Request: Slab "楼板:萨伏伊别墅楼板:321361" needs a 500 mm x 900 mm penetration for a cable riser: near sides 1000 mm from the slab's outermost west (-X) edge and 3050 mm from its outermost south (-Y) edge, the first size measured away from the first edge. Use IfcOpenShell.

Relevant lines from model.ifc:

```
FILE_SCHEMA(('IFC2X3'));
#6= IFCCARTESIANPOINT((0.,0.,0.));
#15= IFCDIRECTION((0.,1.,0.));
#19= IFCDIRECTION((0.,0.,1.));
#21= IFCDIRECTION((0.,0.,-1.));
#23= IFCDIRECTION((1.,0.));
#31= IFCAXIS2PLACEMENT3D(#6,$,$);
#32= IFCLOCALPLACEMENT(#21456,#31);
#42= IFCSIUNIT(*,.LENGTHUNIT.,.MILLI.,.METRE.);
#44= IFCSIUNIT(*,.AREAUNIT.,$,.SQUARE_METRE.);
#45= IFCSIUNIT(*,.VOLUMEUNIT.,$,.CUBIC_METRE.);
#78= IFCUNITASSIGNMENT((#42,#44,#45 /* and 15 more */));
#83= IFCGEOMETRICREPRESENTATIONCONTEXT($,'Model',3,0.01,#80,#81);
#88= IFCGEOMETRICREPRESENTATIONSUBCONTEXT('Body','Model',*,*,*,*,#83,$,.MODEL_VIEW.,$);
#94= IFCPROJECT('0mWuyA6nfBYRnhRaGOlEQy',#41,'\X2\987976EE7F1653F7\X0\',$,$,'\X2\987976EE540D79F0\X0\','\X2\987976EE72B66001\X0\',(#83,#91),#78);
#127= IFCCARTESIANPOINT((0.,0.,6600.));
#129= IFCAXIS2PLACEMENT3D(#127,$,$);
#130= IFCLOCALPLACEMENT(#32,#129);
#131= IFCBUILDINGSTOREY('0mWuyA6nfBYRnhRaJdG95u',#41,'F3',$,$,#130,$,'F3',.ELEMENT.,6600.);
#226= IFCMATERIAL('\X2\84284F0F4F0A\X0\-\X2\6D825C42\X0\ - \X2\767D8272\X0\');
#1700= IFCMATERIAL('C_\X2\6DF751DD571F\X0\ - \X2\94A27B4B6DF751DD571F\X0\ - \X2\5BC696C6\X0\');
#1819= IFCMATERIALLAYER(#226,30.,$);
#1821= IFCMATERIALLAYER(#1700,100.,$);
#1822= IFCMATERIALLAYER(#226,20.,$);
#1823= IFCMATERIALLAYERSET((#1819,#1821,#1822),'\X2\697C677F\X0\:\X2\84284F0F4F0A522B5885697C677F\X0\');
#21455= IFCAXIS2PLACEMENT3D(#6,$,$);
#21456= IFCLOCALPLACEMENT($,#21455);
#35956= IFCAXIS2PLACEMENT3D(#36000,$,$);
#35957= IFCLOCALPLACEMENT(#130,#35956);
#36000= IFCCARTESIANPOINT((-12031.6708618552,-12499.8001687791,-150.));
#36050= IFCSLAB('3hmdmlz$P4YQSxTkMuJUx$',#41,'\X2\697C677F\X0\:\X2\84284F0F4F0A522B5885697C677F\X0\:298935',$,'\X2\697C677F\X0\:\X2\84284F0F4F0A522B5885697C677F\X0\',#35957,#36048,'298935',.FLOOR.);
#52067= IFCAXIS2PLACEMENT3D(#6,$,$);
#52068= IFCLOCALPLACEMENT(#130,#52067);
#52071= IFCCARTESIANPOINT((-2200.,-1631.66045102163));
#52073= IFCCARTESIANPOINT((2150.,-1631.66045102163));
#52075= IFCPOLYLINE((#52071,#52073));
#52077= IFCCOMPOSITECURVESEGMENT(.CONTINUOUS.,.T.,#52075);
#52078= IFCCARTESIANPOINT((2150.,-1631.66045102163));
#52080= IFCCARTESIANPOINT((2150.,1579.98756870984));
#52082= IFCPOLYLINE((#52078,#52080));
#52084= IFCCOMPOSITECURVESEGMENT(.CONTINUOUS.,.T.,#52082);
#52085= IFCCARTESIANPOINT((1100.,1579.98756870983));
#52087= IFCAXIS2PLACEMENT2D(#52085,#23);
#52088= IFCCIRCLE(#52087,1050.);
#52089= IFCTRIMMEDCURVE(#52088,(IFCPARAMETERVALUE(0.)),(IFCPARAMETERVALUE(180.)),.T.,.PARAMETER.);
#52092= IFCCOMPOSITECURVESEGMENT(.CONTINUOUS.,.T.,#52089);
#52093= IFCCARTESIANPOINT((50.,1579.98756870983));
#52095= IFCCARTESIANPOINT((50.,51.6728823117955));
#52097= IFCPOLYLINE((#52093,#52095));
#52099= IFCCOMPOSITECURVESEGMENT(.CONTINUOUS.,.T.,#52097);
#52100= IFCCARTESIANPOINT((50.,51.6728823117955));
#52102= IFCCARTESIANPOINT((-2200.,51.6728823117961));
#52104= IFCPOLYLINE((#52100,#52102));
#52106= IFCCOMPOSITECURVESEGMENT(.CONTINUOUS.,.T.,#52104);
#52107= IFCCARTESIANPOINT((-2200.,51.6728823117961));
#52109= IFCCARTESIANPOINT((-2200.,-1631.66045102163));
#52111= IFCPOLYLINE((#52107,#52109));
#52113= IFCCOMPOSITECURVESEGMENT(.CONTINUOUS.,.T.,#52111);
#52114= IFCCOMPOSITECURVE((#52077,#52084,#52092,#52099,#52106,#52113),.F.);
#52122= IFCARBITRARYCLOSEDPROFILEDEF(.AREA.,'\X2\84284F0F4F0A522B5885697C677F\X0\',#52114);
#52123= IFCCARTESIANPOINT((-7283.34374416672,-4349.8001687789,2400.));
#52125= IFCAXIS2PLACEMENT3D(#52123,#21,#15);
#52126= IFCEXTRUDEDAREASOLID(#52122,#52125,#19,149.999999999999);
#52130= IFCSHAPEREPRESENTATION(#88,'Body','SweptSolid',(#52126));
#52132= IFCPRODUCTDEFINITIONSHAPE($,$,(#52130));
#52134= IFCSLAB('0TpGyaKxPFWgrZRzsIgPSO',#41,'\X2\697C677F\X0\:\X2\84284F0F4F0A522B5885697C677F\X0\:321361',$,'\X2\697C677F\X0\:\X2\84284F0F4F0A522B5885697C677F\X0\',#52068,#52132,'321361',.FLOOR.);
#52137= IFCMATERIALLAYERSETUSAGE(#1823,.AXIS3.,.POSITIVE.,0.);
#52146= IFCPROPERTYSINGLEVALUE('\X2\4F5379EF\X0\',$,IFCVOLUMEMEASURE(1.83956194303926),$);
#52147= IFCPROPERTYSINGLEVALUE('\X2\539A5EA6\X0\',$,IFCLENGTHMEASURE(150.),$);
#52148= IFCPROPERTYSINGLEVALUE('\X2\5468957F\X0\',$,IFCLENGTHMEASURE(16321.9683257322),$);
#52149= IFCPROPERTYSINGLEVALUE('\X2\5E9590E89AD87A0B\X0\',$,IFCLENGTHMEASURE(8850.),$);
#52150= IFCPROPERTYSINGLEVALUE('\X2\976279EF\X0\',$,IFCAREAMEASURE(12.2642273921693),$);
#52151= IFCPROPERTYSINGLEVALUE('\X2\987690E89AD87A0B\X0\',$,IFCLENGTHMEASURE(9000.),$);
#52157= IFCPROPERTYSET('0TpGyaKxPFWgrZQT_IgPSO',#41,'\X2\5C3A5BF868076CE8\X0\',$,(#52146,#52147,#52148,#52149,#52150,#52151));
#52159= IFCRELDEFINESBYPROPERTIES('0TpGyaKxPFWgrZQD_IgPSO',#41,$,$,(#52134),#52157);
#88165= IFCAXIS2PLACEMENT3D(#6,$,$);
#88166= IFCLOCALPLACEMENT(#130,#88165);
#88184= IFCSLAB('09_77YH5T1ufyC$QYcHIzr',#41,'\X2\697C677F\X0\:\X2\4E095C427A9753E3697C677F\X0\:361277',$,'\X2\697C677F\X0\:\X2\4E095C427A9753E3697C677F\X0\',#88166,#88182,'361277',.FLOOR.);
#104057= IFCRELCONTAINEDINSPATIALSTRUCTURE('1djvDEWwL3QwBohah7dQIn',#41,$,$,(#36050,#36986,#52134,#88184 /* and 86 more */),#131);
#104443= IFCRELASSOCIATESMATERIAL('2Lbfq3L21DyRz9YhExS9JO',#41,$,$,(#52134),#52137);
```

```python
import numpy as np
import ifcopenshell
import ifcopenshell.api.feature
import ifcopenshell.api.geometry
import ifcopenshell.api.pset
import ifcopenshell.api.root
import ifcopenshell.geom
import ifcopenshell.util.element
import ifcopenshell.util.placement
import ifcopenshell.util.representation
import ifcopenshell.util.shape
import ifcopenshell.util.unit

model = ifcopenshell.open("model.ifc")
unit_scale = ifcopenshell.util.unit.calculate_unit_scale(model)
area_scale = ifcopenshell.util.unit.calculate_unit_scale(model, "AREAUNIT")
volume_scale = ifcopenshell.util.unit.calculate_unit_scale(model, "VOLUMEUNIT")
settings = ifcopenshell.geom.settings()


def volume(element):
    """Net volume in cubic metres, openings subtracted."""
    shape = ifcopenshell.geom.create_shape(settings, element)
    return ifcopenshell.util.shape.get_volume(shape.geometry)


slab = model.by_guid("0TpGyaKxPFWgrZRzsIgPSO")
before = volume(slab)

# Extent in the slab's own axes, in metres. The edges named are its -X and -Y sides.
slab_shape = ifcopenshell.geom.create_shape(settings, slab)
vertices = ifcopenshell.util.shape.get_vertices(slab_shape.geometry)
x_min, y_min, bottom = vertices.min(axis=0)
top = vertices[:, 2].max()

opening = ifcopenshell.api.root.create_entity(model, ifc_class="IfcOpeningElement", name="Cable riser opening")
context = ifcopenshell.util.representation.get_context(model, "Model", "Body", "MODEL_VIEW")
width, depth = 0.5, 0.9
outline = [(0.0, 0.0), (width, 0.0), (width, depth), (0.0, depth), (0.0, 0.0)]
# Overshoot both faces by 50 mm so the cut is clean.
shape = ifcopenshell.api.geometry.add_slab_representation(
    model, context=context, depth=top - bottom + 0.1, polyline=outline
)
ifcopenshell.api.geometry.assign_representation(model, product=opening, representation=shape)

matrix = ifcopenshell.util.placement.get_local_placement(slab.ObjectPlacement)
matrix[:, 3] = matrix @ np.append(np.array([x_min + 1, y_min + 3.05, bottom - 0.05]) / unit_scale, 1.0)
ifcopenshell.api.geometry.edit_object_placement(model, product=opening, matrix=matrix, is_si=False)
ifcopenshell.api.feature.add_feature(model, feature=opening, element=slab)

after = volume(slab)

# Update the slab's stored quantities.
pset = model.by_id(ifcopenshell.util.element.get_pset(slab, "尺寸标注", should_inherit=False)["id"])
ifcopenshell.api.pset.edit_pset(model, pset=pset, properties={
    "体积": model.create_entity("IfcVolumeMeasure", after / volume_scale),
    "面积": model.create_entity("IfcAreaMeasure", after / (top - bottom) / area_scale),
})

print(f"slab volume {before:.3f} -> {after:.3f} m3")

model.write("model_updated.ifc")
```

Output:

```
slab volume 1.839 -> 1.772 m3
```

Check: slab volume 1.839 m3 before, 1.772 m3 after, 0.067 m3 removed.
